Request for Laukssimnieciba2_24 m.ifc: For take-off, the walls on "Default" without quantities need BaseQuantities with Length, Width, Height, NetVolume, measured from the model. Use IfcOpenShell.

First a look at what the model holds.

```python
import ifcopenshell
import ifcopenshell.util.element
import ifcopenshell.util.unit

model = ifcopenshell.open("Laukssimnieciba2_24 m.ifc")
print(model.schema)
for unit_type in ("LENGTHUNIT", "AREAUNIT", "VOLUMEUNIT"):
    print(unit_type, ifcopenshell.util.unit.calculate_unit_scale(model, unit_type))
storey = next(s for s in model.by_type("IfcBuildingStorey") if s.Name == "Default")
walls = [e for e in ifcopenshell.util.element.get_decomposition(storey) if e.is_a("IfcWall")]
for e in sorted(walls, key=lambda e: e.id()):
    print(e.id(), e.is_a(), e.Name, list(ifcopenshell.util.element.get_psets(e, qtos_only=True)), sep=" | ")
```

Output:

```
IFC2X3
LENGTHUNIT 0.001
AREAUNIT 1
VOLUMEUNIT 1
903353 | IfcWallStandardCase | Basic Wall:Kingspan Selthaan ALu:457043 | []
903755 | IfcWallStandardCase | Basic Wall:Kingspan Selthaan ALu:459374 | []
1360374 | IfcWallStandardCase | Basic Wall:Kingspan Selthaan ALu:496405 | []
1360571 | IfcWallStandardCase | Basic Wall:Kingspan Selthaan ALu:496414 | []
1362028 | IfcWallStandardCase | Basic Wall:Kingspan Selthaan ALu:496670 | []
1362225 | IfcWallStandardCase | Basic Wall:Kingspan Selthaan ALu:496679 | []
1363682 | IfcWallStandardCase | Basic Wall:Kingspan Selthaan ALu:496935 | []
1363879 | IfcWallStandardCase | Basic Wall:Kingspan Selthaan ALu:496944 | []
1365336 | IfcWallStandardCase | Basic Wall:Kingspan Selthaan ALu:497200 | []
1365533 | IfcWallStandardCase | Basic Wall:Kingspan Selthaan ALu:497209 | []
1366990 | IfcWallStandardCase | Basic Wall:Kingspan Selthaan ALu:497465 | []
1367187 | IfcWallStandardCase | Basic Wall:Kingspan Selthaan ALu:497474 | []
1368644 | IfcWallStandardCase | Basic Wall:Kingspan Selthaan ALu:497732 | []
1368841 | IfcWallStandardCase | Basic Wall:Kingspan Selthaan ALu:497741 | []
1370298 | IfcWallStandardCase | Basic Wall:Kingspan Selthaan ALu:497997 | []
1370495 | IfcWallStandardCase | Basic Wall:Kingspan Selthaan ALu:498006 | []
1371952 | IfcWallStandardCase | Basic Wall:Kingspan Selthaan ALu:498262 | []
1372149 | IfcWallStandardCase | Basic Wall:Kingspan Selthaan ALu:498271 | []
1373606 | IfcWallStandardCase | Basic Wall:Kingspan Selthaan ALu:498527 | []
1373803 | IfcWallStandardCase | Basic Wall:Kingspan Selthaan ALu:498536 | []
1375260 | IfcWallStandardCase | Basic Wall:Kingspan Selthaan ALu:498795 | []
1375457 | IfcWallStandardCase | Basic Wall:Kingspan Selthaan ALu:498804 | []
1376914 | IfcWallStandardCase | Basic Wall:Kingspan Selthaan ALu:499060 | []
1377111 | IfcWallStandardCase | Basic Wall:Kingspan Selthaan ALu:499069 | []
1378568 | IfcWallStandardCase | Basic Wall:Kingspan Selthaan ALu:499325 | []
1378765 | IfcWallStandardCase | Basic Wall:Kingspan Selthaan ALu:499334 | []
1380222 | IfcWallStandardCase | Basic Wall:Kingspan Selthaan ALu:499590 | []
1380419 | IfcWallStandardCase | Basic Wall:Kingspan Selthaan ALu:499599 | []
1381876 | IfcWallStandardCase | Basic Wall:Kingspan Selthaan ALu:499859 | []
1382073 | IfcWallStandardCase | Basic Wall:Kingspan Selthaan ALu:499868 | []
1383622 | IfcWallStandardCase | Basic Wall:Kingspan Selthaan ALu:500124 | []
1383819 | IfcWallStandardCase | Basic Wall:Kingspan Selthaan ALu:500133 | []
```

```python
import ifcopenshell
import ifcopenshell.api.pset
import ifcopenshell.geom
import ifcopenshell.util.element
import ifcopenshell.util.shape
import ifcopenshell.util.unit

model = ifcopenshell.open("Laukssimnieciba2_24 m.ifc")
unit_scale = ifcopenshell.util.unit.calculate_unit_scale(model)
volume_scale = ifcopenshell.util.unit.calculate_unit_scale(model, "VOLUMEUNIT")
settings = ifcopenshell.geom.settings()

storey = next(s for s in model.by_type("IfcBuildingStorey") if s.Name == "Default")
walls = [e for e in ifcopenshell.util.element.get_decomposition(storey) if e.is_a("IfcWall")]

for e in sorted(walls, key=lambda e: e.id()):
    if ifcopenshell.util.element.get_psets(e, qtos_only=True, should_inherit=False):
        continue
    # Geometry comes back in metres, in the element's own axes.
    shape = ifcopenshell.geom.create_shape(settings, e)
    values = {
        "Length": ifcopenshell.util.shape.get_x(shape.geometry) / unit_scale,
        "Width": ifcopenshell.util.shape.get_y(shape.geometry) / unit_scale,
        "Height": ifcopenshell.util.shape.get_z(shape.geometry) / unit_scale,
        "NetVolume": ifcopenshell.util.shape.get_volume(shape.geometry) / volume_scale,
    }
    qto = ifcopenshell.api.pset.add_qto(model, product=e, name="BaseQuantities")
    ifcopenshell.api.pset.edit_qto(model, qto=qto, properties=values)
    print(e.id(), {k: round(v, 3) for k, v in values.items()})

model.write("Laukssimnieciba2_24 m_updated.ifc")
```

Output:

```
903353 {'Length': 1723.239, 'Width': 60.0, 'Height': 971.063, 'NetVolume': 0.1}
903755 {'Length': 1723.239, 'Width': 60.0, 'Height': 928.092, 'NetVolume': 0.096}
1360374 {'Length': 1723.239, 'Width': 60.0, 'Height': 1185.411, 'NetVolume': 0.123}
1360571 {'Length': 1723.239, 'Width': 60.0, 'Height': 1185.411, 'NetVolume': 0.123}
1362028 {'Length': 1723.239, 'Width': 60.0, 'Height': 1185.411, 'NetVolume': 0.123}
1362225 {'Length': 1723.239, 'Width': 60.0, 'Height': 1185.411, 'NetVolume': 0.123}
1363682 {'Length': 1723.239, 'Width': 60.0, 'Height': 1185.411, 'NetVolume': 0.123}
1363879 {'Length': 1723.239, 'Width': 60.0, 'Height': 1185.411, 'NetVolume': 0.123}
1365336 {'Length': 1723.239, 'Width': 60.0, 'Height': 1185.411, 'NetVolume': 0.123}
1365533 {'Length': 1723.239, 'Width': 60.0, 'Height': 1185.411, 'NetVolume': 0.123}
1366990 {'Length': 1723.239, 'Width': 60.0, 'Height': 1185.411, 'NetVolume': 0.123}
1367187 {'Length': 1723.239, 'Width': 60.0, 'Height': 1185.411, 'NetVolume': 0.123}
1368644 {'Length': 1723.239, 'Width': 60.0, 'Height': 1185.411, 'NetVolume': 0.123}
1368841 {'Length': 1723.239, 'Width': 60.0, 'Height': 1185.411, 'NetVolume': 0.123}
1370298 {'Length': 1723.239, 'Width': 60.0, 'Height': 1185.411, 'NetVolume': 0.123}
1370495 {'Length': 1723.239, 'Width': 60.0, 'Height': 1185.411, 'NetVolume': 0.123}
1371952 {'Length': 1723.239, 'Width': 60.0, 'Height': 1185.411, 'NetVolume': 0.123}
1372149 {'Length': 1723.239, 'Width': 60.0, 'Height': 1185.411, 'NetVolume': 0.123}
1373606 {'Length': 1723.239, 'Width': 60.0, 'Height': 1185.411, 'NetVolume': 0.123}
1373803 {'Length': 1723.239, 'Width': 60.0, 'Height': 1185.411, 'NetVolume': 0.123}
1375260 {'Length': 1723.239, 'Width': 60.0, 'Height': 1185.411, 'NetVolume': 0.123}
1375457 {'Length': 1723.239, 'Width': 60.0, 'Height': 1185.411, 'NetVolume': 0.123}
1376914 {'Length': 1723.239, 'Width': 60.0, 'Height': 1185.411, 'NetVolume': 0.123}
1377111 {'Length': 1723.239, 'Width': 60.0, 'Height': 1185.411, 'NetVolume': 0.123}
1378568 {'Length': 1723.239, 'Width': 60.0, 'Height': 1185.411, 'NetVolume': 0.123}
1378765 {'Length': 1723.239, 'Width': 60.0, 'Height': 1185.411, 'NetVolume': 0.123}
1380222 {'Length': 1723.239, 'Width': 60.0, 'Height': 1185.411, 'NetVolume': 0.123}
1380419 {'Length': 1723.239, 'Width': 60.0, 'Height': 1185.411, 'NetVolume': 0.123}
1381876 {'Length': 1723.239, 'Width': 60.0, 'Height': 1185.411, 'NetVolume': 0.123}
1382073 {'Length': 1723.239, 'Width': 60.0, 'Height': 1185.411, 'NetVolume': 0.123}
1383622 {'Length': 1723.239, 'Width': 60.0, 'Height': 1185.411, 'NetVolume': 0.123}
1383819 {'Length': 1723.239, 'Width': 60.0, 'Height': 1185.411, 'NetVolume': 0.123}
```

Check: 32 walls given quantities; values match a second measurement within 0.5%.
